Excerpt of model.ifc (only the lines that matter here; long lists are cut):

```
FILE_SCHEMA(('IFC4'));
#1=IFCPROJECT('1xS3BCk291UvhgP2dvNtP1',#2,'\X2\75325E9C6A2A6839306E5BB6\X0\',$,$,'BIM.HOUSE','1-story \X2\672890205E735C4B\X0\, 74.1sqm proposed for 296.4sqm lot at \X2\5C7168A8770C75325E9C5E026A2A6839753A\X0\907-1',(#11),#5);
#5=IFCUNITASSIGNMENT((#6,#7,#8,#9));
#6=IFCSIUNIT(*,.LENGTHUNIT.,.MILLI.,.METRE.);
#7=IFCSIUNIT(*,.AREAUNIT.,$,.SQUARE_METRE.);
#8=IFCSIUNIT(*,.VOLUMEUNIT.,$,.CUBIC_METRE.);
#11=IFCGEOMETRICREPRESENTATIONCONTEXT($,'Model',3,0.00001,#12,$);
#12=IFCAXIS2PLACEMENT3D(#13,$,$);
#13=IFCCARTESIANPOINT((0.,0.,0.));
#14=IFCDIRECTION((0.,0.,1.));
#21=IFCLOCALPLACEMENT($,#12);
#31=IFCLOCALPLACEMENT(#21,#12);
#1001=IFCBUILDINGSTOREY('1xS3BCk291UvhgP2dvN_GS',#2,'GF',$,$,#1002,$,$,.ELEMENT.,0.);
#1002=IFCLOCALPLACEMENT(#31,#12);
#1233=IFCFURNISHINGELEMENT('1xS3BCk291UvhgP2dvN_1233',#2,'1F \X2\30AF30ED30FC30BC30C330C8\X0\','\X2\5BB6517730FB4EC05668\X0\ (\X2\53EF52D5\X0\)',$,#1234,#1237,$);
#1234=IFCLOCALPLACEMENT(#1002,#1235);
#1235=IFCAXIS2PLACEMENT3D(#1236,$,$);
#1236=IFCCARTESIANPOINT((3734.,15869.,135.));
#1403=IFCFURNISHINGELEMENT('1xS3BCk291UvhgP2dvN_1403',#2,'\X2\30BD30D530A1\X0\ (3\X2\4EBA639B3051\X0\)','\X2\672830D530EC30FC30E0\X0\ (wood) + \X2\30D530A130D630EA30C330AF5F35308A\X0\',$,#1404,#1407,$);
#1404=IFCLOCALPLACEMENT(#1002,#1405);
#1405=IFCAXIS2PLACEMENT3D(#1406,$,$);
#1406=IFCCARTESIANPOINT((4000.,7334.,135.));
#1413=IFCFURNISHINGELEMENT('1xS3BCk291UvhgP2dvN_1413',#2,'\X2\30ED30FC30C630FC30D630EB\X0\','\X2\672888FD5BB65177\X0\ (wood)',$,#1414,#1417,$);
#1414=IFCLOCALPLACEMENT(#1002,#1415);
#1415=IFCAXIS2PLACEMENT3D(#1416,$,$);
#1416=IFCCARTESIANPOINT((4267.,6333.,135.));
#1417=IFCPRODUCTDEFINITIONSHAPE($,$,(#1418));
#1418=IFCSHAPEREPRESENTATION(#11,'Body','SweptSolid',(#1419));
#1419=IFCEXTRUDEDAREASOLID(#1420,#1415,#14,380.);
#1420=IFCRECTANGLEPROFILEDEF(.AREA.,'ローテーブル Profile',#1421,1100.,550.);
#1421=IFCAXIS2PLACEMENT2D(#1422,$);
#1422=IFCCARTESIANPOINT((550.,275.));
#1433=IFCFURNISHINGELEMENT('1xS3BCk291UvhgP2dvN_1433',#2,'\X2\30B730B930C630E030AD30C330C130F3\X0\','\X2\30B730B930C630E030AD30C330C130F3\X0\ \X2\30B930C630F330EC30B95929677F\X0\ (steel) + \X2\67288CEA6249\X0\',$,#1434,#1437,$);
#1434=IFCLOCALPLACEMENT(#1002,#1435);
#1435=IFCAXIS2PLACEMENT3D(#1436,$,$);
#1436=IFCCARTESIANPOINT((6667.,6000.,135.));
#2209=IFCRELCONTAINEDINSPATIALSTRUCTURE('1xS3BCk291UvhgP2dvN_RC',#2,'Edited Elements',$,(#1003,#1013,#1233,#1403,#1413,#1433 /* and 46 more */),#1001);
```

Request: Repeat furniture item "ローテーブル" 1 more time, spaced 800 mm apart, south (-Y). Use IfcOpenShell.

```python
import numpy as np
import ifcopenshell
import ifcopenshell.api.geometry
import ifcopenshell.api.root
import ifcopenshell.util.element
import ifcopenshell.util.placement
import ifcopenshell.util.unit

model = ifcopenshell.open("model.ifc")
unit_scale = ifcopenshell.util.unit.calculate_unit_scale(model)


def reuse_history(source, copy):
    """copy_class also copies each property set's owner history, people and application; keep the originals."""
    for rel in copy.IsDefinedBy:
        if rel.is_a("IfcRelDefinesByProperties") and (history := rel.RelatingPropertyDefinition.OwnerHistory):
            rel.RelatingPropertyDefinition.OwnerHistory = source.OwnerHistory
            ifcopenshell.util.element.remove_deep2(model, history)


source = model.by_guid("1xS3BCk291UvhgP2dvN_1413")
base = ifcopenshell.util.placement.get_local_placement(source.ObjectPlacement)
step = np.array([0.0, -1.0, 0.0]) * 0.8 / unit_scale

for i in range(1, 2):
    copy = ifcopenshell.api.root.copy_class(model, product=source)
    copy.Representation = ifcopenshell.util.element.copy_deep(
        model, source.Representation, exclude=["IfcGeometricRepresentationContext", "IfcRepresentationMap"]
    )
    reuse_history(source, copy)
    matrix = base.copy()
    matrix[:3, 3] += i * step
    print("added at", matrix[:3, 3].round(3) + 0.0)
    ifcopenshell.api.geometry.edit_object_placement(model, product=copy, matrix=matrix, is_si=False)

model.write("model_edited.ifc")
```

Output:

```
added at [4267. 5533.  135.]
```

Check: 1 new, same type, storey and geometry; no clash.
